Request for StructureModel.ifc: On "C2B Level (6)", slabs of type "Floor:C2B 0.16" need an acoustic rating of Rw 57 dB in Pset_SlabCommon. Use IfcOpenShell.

First a look at what the model holds.

```python
import ifcopenshell
import ifcopenshell.util.element

model = ifcopenshell.open("StructureModel.ifc")
print(model.schema)
storey = next(s for s in model.by_type("IfcBuildingStorey") if s.Name == "C2B Level (6)")
slabs = [e for e in ifcopenshell.util.element.get_decomposition(storey) if e.is_a("IfcSlab")]
seen = {}
for e in slabs:
    element_type = ifcopenshell.util.element.get_type(e)
    key = (element_type.Name if element_type != e and element_type else None, ifcopenshell.util.element.get_pset(e, "Pset_SlabCommon", "AcousticRating"))
    seen[key] = seen.get(key, 0) + 1
for (name, value), count in sorted(seen.items(), key=str):
    print(count, "x", name, "|", value)
```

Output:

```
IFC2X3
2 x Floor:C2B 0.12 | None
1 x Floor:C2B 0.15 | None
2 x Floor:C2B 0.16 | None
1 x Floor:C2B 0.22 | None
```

```python
import ifcopenshell
import ifcopenshell.api.pset
import ifcopenshell.util.element

model = ifcopenshell.open("StructureModel.ifc")

storey = next(s for s in model.by_type("IfcBuildingStorey") if s.Name == "C2B Level (6)")
slabs = [e for e in ifcopenshell.util.element.get_decomposition(storey) if e.is_a("IfcSlab")]

count = 0
for e in slabs:
    element_type = ifcopenshell.util.element.get_type(e)
    if element_type in (None, e) or element_type.Name != "Floor:C2B 0.16":
        continue
    # add_pset returns the element's existing set when there is one.
    pset = ifcopenshell.api.pset.add_pset(model, product=e, name="Pset_SlabCommon")
    ifcopenshell.api.pset.edit_pset(model, pset=pset, properties={"AcousticRating": "Rw 57 dB"})
    count += 1

print(count, "slabs updated")

model.write("StructureModel_v2.ifc")
```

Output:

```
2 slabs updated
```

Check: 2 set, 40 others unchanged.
